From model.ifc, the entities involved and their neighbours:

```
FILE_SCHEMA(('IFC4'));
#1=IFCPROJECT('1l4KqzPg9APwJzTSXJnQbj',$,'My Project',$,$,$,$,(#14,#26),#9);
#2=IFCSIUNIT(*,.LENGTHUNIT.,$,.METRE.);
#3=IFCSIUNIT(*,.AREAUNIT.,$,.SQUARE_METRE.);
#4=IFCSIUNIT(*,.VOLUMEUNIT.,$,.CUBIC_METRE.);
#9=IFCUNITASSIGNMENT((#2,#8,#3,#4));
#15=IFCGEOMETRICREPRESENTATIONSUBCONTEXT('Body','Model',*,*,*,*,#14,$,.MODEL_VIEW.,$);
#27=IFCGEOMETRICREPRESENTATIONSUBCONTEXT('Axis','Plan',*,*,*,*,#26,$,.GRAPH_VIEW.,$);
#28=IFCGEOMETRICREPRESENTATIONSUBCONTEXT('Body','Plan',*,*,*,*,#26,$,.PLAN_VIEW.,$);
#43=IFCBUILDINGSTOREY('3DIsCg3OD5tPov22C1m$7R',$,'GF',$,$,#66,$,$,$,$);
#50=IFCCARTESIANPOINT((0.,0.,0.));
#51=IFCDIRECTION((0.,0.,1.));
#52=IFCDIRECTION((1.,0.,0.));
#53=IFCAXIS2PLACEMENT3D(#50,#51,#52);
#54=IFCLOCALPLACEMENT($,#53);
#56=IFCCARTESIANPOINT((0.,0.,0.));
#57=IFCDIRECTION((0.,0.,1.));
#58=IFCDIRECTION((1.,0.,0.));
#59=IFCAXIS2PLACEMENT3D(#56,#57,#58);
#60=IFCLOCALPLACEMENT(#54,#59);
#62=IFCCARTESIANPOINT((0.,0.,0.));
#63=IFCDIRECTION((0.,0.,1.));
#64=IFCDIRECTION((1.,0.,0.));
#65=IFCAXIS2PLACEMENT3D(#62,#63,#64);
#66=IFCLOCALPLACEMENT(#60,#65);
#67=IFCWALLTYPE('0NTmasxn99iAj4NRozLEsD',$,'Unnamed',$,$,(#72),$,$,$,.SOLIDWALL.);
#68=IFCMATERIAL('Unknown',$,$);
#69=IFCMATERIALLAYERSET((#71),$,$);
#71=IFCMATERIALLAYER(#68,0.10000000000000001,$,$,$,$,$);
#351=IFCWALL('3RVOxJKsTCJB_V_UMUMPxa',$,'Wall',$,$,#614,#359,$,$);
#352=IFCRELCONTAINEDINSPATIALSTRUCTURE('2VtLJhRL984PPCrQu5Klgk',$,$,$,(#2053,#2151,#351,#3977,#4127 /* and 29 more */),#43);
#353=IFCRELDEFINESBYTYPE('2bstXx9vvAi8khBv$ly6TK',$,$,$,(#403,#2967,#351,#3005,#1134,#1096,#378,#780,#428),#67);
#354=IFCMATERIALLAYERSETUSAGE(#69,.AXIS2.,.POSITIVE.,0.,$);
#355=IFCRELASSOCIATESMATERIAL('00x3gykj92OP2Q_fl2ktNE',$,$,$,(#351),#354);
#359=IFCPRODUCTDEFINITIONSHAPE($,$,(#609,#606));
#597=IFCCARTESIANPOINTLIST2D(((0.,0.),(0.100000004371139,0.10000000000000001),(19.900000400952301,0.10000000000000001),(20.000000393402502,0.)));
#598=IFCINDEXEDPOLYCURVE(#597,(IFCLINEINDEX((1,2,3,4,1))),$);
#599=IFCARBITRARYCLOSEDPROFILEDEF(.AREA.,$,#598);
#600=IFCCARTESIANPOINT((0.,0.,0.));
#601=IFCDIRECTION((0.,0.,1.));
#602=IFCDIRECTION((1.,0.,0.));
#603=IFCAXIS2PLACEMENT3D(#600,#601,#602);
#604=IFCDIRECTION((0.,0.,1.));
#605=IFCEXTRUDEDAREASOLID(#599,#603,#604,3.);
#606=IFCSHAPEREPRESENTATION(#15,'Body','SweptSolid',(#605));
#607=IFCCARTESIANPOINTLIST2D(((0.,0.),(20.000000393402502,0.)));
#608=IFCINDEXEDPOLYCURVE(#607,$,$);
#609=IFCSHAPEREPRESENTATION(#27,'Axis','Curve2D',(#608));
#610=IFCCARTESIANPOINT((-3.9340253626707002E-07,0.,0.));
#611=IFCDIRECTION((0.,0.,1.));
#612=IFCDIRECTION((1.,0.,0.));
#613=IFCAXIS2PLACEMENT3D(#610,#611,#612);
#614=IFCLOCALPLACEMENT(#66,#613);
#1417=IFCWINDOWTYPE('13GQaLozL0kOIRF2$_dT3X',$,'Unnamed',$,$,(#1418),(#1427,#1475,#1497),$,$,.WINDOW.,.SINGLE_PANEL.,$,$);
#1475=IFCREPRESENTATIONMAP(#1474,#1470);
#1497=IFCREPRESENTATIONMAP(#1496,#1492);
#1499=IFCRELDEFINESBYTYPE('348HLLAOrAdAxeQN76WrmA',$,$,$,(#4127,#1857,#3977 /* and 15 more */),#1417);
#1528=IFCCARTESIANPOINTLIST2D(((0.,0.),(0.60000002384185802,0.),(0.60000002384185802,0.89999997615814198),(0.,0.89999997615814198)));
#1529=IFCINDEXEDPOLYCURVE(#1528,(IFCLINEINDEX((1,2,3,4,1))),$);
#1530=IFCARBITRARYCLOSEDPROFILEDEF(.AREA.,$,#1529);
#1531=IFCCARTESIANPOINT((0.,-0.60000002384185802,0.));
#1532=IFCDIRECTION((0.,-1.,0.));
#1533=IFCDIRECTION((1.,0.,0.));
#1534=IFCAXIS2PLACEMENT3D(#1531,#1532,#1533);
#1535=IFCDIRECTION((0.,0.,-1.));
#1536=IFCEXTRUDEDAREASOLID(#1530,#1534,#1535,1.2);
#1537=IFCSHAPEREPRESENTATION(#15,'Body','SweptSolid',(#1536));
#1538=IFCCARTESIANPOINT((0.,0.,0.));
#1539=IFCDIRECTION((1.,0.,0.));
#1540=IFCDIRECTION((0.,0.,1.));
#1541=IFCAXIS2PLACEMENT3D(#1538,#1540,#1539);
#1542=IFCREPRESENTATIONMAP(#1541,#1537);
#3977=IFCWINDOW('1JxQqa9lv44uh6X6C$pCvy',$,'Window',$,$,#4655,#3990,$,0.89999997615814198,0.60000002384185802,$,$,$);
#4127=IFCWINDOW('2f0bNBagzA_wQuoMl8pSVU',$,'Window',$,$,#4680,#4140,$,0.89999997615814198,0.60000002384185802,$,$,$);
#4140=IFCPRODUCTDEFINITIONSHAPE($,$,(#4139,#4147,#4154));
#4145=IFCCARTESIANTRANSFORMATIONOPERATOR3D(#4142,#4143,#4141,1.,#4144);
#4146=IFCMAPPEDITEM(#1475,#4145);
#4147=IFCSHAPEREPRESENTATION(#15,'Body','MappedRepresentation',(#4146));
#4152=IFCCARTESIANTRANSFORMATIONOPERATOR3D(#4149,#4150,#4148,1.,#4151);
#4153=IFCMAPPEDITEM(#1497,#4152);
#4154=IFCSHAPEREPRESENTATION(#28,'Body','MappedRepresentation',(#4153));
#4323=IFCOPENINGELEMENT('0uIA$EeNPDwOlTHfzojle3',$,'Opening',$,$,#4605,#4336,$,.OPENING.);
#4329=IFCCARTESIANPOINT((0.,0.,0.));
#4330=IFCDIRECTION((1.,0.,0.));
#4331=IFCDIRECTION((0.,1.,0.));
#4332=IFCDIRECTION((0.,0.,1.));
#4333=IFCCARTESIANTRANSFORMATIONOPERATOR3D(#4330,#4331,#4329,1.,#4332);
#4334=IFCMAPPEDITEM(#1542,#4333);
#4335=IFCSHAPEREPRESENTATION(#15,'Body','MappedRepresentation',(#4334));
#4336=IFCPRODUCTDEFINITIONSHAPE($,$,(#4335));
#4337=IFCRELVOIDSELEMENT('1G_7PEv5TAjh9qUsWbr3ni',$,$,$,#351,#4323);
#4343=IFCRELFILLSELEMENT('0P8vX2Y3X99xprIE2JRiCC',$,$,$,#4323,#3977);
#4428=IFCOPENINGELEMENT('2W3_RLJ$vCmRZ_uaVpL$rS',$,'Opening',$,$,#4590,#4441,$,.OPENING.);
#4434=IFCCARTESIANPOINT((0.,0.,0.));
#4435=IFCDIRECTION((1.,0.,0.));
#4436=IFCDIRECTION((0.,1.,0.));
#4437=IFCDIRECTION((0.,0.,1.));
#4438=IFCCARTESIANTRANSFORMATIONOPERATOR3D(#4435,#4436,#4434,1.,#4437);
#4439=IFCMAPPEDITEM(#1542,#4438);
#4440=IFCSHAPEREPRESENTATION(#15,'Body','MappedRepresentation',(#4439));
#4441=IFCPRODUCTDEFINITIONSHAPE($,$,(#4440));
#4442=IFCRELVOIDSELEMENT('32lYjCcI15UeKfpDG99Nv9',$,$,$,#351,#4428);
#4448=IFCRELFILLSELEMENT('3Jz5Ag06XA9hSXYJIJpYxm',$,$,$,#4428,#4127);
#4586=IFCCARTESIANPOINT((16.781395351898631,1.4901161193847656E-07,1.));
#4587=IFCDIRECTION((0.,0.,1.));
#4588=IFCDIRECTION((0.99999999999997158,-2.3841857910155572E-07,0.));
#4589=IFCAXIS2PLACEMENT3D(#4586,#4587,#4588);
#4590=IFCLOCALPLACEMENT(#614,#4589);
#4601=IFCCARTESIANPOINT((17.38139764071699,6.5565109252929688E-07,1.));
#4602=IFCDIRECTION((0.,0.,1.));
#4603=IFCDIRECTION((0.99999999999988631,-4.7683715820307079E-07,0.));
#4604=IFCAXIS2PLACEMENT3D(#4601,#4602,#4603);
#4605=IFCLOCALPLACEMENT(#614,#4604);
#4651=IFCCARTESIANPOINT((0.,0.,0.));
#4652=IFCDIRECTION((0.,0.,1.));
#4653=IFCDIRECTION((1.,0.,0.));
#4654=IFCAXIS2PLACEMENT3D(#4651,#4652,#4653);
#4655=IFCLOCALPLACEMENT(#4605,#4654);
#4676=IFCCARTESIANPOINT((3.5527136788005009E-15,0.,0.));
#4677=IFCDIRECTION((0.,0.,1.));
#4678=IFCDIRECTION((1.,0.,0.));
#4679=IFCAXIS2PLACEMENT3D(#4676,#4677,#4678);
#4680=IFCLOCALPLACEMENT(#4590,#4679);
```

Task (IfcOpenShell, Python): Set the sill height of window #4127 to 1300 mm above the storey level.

```python
import numpy as np
import ifcopenshell
import ifcopenshell.api.geometry
import ifcopenshell.geom
import ifcopenshell.util.element
import ifcopenshell.util.placement
import ifcopenshell.util.shape
import ifcopenshell.util.unit

model = ifcopenshell.open("model.ifc")
unit_scale = ifcopenshell.util.unit.calculate_unit_scale(model)

window = model.by_guid("2f0bNBagzA_wQuoMl8pSVU")
opening = window.FillsVoids[0].RelatingOpeningElement
storey = ifcopenshell.util.element.get_container(window, ifc_class="IfcBuildingStorey")
level = ifcopenshell.util.placement.get_local_placement(storey.ObjectPlacement)[2, 3]

# The opening's origin need not be at the sill, so measure its lowest point.
shape = ifcopenshell.geom.create_shape(ifcopenshell.geom.settings(), opening)
bottom = ifcopenshell.util.shape.get_shape_bottom_elevation(shape, shape.geometry) / unit_scale
dz = level + 1.3 / unit_scale - bottom

shift = np.array([0.0, 0.0, dz])
# The window is placed relative to its opening, so it follows when the opening moves.
matrix = ifcopenshell.util.placement.get_local_placement(opening.ObjectPlacement)
matrix[:3, 3] += shift
ifcopenshell.api.geometry.edit_object_placement(
    model, product=opening, matrix=matrix, is_si=False, should_transform_children=True
)

print(f"moved by {dz * unit_scale:+.3f} m")

model.write("model-out.ifc")
```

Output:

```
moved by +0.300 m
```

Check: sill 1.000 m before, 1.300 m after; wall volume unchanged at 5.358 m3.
